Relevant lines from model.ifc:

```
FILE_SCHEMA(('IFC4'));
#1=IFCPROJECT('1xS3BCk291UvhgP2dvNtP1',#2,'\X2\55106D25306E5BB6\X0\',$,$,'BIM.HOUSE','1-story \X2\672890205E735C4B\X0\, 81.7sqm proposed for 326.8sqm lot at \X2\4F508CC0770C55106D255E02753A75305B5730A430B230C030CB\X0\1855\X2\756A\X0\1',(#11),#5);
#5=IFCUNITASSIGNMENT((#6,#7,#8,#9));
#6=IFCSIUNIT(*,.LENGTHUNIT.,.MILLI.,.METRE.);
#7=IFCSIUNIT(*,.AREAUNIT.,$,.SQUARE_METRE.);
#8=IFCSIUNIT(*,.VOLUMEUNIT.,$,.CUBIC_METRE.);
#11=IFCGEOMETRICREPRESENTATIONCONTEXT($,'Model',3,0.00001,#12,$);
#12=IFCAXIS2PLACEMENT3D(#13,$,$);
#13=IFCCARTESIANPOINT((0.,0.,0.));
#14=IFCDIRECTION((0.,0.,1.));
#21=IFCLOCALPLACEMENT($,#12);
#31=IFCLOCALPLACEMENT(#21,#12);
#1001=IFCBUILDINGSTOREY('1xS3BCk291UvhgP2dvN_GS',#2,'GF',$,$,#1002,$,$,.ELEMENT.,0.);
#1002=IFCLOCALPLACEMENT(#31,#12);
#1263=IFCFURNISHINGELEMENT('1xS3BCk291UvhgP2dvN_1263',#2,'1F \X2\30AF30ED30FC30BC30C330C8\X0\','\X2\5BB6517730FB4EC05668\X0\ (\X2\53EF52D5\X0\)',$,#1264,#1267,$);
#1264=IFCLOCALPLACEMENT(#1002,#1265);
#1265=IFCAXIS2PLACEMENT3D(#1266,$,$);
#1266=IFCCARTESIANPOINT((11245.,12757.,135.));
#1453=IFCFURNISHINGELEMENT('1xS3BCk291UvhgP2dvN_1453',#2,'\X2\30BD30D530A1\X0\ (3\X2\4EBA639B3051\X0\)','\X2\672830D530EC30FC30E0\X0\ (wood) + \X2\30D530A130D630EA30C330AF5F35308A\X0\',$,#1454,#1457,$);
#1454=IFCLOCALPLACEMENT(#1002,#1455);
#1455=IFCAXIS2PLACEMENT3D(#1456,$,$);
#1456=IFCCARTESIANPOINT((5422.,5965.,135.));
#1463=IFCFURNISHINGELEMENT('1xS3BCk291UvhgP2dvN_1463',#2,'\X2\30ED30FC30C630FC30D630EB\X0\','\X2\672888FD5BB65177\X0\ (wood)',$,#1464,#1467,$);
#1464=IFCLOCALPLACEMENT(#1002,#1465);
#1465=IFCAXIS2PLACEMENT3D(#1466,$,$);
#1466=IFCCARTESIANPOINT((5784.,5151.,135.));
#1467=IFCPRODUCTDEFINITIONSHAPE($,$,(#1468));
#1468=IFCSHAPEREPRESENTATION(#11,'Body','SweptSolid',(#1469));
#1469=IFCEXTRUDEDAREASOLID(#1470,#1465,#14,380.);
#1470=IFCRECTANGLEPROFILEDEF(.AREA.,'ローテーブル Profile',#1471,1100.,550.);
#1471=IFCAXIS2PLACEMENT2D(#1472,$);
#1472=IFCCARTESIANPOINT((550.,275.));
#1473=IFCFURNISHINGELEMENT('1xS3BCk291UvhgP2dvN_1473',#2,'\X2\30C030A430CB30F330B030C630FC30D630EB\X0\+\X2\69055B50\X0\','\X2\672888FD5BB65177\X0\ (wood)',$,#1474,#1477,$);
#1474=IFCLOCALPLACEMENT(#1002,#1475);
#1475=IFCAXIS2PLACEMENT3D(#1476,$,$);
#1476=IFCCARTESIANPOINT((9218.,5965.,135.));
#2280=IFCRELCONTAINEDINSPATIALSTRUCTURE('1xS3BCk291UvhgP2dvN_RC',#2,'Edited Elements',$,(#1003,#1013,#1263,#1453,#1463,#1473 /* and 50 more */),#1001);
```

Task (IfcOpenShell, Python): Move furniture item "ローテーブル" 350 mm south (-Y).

```python
import ifcopenshell
import ifcopenshell.api.geometry
import ifcopenshell.util.placement

model = ifcopenshell.open("model.ifc")

item = model.by_guid("1xS3BCk291UvhgP2dvN_1463")
matrix = ifcopenshell.util.placement.get_local_placement(item.ObjectPlacement)
matrix[1, 3] -= 350.0
ifcopenshell.api.geometry.edit_object_placement(model, product=item, matrix=matrix, is_si=False)

print(ifcopenshell.util.placement.get_local_placement(item.ObjectPlacement).round(3) + 0.0)

model.write("model_rev.ifc")
```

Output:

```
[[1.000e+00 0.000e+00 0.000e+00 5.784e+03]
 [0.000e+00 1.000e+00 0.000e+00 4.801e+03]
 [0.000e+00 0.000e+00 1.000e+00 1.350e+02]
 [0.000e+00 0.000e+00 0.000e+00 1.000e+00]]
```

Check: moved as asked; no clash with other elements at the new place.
